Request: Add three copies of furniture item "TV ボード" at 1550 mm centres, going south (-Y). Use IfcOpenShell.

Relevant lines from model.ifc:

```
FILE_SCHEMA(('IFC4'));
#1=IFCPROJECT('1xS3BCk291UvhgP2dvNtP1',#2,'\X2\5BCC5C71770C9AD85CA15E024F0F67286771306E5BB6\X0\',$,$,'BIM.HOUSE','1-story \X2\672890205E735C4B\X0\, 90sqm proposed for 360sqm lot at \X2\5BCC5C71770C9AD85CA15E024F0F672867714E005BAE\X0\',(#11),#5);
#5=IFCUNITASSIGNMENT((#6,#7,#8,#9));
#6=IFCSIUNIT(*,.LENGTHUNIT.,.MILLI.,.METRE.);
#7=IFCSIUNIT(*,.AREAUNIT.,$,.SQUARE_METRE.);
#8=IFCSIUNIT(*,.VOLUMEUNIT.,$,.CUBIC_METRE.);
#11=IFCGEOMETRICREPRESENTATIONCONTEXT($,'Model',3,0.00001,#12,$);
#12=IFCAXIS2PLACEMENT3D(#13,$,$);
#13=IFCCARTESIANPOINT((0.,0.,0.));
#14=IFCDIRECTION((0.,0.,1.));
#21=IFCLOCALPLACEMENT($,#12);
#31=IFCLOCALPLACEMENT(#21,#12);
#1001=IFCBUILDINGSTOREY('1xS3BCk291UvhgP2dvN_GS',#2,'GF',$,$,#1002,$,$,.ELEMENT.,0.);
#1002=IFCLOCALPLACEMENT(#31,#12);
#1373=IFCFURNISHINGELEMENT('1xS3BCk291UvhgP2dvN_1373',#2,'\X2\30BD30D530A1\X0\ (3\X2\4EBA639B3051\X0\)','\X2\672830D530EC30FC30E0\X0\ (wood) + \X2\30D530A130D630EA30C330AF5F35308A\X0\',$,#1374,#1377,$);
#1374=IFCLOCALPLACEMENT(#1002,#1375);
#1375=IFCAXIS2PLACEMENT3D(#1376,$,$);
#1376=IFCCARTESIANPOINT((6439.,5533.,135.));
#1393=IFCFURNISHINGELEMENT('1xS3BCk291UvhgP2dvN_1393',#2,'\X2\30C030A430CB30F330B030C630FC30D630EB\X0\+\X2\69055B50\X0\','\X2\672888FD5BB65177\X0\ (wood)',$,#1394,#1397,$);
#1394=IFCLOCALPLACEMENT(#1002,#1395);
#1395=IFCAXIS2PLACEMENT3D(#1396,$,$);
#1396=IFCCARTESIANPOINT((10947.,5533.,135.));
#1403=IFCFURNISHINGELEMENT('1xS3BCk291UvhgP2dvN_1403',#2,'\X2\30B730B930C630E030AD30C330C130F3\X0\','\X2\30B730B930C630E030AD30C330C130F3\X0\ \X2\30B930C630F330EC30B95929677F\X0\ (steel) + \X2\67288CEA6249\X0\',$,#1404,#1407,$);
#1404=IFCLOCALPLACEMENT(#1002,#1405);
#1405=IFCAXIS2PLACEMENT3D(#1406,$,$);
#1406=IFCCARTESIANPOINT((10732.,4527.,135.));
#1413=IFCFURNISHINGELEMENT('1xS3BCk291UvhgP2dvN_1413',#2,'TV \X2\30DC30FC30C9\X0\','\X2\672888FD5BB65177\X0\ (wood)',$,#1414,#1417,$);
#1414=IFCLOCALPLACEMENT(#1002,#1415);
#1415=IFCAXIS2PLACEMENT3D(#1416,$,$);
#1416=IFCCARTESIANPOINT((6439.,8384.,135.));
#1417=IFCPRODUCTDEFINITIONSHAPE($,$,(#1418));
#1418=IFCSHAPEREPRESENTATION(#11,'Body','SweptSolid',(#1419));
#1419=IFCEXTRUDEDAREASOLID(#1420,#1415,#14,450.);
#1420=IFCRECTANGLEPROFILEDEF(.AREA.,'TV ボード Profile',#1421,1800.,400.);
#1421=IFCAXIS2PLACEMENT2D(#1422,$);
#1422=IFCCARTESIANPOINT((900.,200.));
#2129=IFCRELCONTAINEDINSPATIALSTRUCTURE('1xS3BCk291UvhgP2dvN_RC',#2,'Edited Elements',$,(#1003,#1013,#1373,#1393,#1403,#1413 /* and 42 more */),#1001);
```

```python
import numpy as np
import ifcopenshell
import ifcopenshell.api.geometry
import ifcopenshell.api.root
import ifcopenshell.util.element
import ifcopenshell.util.placement

model = ifcopenshell.open("model.ifc")


def reuse_history(source, copy):
    """copy_class also copies each property set's owner history, people and application; keep the originals."""
    for rel in copy.IsDefinedBy:
        if rel.is_a("IfcRelDefinesByProperties") and (history := rel.RelatingPropertyDefinition.OwnerHistory):
            rel.RelatingPropertyDefinition.OwnerHistory = source.OwnerHistory
            ifcopenshell.util.element.remove_deep2(model, history)


source = model.by_guid("1xS3BCk291UvhgP2dvN_1413")
base = ifcopenshell.util.placement.get_local_placement(source.ObjectPlacement)
step = np.array([0.0, -1.0, 0.0]) * 1550.0

for i in range(1, 4):
    copy = ifcopenshell.api.root.copy_class(model, product=source)
    copy.Representation = ifcopenshell.util.element.copy_deep(
        model, source.Representation, exclude=["IfcGeometricRepresentationContext", "IfcRepresentationMap"]
    )
    reuse_history(source, copy)
    matrix = base.copy()
    matrix[:3, 3] += i * step
    print("added at", matrix[:3, 3].round(3) + 0.0)
    ifcopenshell.api.geometry.edit_object_placement(model, product=copy, matrix=matrix, is_si=False)

model.write("model-out.ifc")
```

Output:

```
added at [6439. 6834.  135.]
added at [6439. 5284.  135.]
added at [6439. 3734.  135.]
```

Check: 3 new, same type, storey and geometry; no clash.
